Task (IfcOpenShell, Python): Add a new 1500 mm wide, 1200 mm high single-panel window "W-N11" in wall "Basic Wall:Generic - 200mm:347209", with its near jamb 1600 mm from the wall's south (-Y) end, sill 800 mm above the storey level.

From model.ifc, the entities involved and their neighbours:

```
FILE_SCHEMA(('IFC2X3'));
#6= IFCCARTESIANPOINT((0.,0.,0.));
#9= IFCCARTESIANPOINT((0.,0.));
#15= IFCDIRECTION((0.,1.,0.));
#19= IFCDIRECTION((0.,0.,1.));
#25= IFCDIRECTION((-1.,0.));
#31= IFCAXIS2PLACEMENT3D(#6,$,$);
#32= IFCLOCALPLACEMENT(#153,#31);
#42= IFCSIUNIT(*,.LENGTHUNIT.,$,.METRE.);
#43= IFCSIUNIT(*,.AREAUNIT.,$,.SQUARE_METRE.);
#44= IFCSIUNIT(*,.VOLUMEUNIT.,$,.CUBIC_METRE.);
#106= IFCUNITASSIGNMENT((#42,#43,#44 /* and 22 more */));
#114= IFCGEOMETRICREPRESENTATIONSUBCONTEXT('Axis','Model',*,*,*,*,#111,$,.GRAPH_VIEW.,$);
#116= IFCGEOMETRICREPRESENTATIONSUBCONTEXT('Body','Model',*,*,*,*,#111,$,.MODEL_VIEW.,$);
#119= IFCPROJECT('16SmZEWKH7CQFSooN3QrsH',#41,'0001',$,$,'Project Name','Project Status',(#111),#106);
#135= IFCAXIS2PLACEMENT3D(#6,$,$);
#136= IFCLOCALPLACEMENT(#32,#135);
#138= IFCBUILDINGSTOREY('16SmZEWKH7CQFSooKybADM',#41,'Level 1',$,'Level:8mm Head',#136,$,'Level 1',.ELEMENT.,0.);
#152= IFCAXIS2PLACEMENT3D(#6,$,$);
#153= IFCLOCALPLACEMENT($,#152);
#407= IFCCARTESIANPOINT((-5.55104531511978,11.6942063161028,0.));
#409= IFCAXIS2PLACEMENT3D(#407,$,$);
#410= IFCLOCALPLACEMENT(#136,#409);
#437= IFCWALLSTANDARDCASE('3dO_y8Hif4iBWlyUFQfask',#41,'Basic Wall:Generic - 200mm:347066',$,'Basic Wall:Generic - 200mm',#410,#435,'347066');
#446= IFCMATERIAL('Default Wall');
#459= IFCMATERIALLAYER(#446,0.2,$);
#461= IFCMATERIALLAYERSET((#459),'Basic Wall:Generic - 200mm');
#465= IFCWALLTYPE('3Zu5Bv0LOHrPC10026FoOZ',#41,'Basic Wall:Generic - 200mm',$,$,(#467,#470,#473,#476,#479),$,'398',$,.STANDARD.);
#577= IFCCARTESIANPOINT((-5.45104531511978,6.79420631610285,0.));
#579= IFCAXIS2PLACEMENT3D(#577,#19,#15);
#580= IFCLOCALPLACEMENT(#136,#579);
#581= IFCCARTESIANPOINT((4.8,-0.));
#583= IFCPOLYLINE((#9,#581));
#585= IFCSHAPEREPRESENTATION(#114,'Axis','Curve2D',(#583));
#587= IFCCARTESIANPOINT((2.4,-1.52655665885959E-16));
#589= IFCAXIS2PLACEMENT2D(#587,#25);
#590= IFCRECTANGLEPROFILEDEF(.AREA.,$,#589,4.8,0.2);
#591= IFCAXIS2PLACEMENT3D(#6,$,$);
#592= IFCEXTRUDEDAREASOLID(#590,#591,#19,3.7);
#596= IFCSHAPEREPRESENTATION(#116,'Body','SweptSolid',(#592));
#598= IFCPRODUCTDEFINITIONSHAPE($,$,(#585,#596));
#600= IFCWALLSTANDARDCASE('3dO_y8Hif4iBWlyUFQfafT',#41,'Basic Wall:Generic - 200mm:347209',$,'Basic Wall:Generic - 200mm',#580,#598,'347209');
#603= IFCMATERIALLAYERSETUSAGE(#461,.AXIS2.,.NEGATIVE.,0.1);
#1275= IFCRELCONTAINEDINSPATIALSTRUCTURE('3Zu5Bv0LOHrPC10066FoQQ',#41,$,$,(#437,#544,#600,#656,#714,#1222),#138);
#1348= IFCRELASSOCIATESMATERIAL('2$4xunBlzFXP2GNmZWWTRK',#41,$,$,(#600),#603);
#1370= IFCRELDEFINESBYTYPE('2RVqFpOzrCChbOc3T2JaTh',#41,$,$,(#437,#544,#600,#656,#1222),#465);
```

```python
import numpy as np
import ifcopenshell
import ifcopenshell.api.feature
import ifcopenshell.api.geometry
import ifcopenshell.api.root
import ifcopenshell.api.spatial
import ifcopenshell.api.type
import ifcopenshell.geom
import ifcopenshell.util.element
import ifcopenshell.util.placement
import ifcopenshell.util.representation
import ifcopenshell.util.shape
import ifcopenshell.util.unit

model = ifcopenshell.open("model.ifc")
unit_scale = ifcopenshell.util.unit.calculate_unit_scale(model)
settings = ifcopenshell.geom.settings()


def volume(element):
    """Net volume in cubic metres, openings subtracted."""
    shape = ifcopenshell.geom.create_shape(settings, element)
    return ifcopenshell.util.shape.get_volume(shape.geometry)


wall = model.by_guid("3dO_y8Hif4iBWlyUFQfafT")
storey = ifcopenshell.util.element.get_container(wall, ifc_class="IfcBuildingStorey")
context = ifcopenshell.util.representation.get_context(model, "Model", "Body", "MODEL_VIEW")
before = volume(wall)

width, height, from_end, sill = 1.5, 1.2, 1.6, 0.8  # metres

# The wall runs along its own X axis, and the end named is its -X end.
wall_shape = ifcopenshell.geom.create_shape(settings, wall)
x, y, z = ifcopenshell.util.shape.get_vertices(wall_shape.geometry).T
start = x.min() + from_end
face, thickness = float(y.min()), float(y.max() - y.min())
wall_matrix = ifcopenshell.util.placement.get_local_placement(wall.ObjectPlacement)
level = ifcopenshell.util.placement.get_local_placement(storey.ObjectPlacement)[2, 3]


def in_wall(x, y):
    """Placement at x, y metres in the wall's axes, at sill height."""
    matrix = wall_matrix.copy()
    matrix[:, 3] = wall_matrix @ np.array([x / unit_scale, y / unit_scale, 0.0, 1.0])
    matrix[2, 3] = level + sill / unit_scale
    return matrix


# Opening: a box that overshoots both wall faces by 50 mm.
opening = ifcopenshell.api.root.create_entity(model, ifc_class="IfcOpeningElement")
box = ifcopenshell.api.geometry.add_wall_representation(
    model, context=context, length=width, height=height, thickness=thickness + 0.1
)
ifcopenshell.api.geometry.assign_representation(model, product=opening, representation=box)
ifcopenshell.api.geometry.edit_object_placement(model, product=opening, matrix=in_wall(start, face - 0.05), is_si=False)
ifcopenshell.api.feature.add_feature(model, feature=opening, element=wall)

window = ifcopenshell.api.root.create_entity(model, ifc_class="IfcWindow", name="W-N11")
window.OverallWidth, window.OverallHeight = width / unit_scale, height / unit_scale
body = ifcopenshell.api.geometry.add_window_representation(
    model,
    context=context,
    overall_width=window.OverallWidth,
    overall_height=window.OverallHeight,
    partition_type="SINGLE_PANEL",
)
ifcopenshell.api.geometry.assign_representation(model, product=window, representation=body)
ifcopenshell.api.spatial.assign_container(model, products=[window], relating_structure=storey)
fills = ifcopenshell.api.feature.add_filling(model, opening=opening, element=window)
fills.OwnerHistory = window.OwnerHistory  # required in IFC2X3

# IFC2X3 keeps the operation on the window style.
style = ifcopenshell.api.root.create_entity(model, ifc_class="IfcWindowStyle", name="W-N11")
style.OperationType, style.ConstructionType = "SINGLE_PANEL", "NOTDEFINED"
style.ParameterTakesPrecedence = style.Sizeable = False
ifcopenshell.api.type.assign_type(model, related_objects=[window], relating_type=style)

# Centre the window in the wall's thickness.
ifcopenshell.api.geometry.edit_object_placement(model, product=window, matrix=in_wall(start, face), is_si=False)
window_shape = ifcopenshell.geom.create_shape(settings, window)
depth = ifcopenshell.util.shape.get_vertices(window_shape.geometry)[:, 1]
offset = face + thickness / 2 - (depth.min() + depth.max()) / 2
ifcopenshell.api.geometry.edit_object_placement(model, product=window, matrix=in_wall(start, offset), is_si=False)

after = volume(wall)

print(f"wall volume {before:.3f} -> {after:.3f} m3")

model.write("model_updated.ifc")
```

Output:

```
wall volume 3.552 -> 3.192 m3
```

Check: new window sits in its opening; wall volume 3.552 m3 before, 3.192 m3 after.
